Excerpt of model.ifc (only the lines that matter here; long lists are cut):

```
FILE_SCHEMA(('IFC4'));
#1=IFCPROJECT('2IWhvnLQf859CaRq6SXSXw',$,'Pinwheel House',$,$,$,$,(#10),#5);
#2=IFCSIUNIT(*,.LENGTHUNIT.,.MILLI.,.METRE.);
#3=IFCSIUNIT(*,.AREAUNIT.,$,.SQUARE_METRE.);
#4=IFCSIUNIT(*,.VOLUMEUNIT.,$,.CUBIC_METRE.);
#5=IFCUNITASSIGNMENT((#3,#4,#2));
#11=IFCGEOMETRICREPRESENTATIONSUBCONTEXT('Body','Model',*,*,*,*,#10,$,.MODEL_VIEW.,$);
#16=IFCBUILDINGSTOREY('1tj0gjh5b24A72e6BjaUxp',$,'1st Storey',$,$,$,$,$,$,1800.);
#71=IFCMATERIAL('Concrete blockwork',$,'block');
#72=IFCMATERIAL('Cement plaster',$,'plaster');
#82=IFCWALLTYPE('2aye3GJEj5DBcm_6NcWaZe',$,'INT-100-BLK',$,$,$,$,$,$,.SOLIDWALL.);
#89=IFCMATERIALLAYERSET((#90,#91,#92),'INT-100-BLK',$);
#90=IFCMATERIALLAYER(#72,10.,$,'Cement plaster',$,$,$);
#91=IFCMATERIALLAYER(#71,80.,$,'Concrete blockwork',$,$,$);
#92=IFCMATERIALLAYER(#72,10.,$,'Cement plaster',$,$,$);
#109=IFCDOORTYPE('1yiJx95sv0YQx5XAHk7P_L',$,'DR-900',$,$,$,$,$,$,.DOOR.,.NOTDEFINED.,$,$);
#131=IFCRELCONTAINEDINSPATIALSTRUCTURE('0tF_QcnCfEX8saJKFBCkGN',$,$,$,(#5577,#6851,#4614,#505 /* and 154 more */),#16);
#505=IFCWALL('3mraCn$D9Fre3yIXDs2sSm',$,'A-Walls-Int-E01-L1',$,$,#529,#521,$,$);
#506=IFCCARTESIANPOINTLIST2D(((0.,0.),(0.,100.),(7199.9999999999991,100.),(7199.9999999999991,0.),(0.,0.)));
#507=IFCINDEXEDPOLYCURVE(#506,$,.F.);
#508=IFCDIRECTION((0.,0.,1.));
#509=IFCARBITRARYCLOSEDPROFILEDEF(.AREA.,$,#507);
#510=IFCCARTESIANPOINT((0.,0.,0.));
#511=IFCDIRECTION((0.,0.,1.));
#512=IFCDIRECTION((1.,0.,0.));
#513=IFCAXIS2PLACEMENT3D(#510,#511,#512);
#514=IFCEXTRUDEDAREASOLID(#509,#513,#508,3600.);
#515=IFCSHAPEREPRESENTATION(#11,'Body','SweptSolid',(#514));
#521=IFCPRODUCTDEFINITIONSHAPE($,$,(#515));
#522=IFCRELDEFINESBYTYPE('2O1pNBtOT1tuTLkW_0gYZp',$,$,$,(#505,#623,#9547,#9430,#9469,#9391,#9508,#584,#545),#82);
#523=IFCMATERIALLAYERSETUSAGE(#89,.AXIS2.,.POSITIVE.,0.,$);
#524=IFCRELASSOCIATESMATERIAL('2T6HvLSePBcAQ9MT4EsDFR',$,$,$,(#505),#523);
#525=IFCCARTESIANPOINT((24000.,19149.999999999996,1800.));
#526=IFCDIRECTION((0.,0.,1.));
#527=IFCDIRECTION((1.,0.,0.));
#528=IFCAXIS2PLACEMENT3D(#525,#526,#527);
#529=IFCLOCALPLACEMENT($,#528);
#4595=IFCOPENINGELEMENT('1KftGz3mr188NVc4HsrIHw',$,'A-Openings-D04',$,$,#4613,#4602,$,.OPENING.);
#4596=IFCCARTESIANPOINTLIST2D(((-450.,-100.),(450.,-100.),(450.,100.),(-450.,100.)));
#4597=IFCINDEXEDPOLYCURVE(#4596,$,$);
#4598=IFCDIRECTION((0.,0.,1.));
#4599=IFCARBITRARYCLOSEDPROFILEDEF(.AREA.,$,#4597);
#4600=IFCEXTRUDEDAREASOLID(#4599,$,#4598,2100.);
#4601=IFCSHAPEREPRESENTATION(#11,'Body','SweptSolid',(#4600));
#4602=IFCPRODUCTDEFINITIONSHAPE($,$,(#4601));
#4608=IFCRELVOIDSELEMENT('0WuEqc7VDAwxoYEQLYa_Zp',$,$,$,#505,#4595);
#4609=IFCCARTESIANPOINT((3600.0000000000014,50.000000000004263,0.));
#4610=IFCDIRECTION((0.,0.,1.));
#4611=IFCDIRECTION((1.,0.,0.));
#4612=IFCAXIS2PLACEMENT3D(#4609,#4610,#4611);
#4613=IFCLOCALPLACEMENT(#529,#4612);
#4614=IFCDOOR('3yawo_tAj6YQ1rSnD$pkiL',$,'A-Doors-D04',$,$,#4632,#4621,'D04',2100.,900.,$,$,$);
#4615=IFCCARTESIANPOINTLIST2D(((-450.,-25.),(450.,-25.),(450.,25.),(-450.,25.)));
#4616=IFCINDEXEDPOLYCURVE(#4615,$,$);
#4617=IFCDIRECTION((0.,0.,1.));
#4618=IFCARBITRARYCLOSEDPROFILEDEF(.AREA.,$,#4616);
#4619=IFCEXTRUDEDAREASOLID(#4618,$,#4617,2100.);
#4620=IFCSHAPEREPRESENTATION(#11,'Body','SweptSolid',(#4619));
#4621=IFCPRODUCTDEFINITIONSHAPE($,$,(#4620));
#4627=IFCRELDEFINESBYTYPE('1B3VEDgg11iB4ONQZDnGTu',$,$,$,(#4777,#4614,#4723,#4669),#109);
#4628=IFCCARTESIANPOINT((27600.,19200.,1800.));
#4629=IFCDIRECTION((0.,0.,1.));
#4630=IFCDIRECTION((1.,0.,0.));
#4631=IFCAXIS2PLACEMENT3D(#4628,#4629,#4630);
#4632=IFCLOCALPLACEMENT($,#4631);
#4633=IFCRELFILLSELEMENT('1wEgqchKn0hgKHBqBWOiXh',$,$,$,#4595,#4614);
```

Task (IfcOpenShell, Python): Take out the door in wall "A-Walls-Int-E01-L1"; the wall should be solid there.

```python
import ifcopenshell
import ifcopenshell.api.feature
import ifcopenshell.api.root
import ifcopenshell.geom
import ifcopenshell.util.shape

model = ifcopenshell.open("model.ifc")
settings = ifcopenshell.geom.settings()


def volume(element):
    """Net volume in cubic metres, openings subtracted."""
    shape = ifcopenshell.geom.create_shape(settings, element)
    return ifcopenshell.util.shape.get_volume(shape.geometry)


door = model.by_id(4614)
opening = door.FillsVoids[0].RelatingOpeningElement
wall = opening.VoidsElements[0].RelatingBuildingElement
before = volume(wall)

ifcopenshell.api.root.remove_product(model, product=door)
ifcopenshell.api.feature.remove_feature(model, feature=opening)

after = volume(wall)

print(f"wall volume {before:.3f} -> {after:.3f} m3")

model.write("model_updated.ifc")
```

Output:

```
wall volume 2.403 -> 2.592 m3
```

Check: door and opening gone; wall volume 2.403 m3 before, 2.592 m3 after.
